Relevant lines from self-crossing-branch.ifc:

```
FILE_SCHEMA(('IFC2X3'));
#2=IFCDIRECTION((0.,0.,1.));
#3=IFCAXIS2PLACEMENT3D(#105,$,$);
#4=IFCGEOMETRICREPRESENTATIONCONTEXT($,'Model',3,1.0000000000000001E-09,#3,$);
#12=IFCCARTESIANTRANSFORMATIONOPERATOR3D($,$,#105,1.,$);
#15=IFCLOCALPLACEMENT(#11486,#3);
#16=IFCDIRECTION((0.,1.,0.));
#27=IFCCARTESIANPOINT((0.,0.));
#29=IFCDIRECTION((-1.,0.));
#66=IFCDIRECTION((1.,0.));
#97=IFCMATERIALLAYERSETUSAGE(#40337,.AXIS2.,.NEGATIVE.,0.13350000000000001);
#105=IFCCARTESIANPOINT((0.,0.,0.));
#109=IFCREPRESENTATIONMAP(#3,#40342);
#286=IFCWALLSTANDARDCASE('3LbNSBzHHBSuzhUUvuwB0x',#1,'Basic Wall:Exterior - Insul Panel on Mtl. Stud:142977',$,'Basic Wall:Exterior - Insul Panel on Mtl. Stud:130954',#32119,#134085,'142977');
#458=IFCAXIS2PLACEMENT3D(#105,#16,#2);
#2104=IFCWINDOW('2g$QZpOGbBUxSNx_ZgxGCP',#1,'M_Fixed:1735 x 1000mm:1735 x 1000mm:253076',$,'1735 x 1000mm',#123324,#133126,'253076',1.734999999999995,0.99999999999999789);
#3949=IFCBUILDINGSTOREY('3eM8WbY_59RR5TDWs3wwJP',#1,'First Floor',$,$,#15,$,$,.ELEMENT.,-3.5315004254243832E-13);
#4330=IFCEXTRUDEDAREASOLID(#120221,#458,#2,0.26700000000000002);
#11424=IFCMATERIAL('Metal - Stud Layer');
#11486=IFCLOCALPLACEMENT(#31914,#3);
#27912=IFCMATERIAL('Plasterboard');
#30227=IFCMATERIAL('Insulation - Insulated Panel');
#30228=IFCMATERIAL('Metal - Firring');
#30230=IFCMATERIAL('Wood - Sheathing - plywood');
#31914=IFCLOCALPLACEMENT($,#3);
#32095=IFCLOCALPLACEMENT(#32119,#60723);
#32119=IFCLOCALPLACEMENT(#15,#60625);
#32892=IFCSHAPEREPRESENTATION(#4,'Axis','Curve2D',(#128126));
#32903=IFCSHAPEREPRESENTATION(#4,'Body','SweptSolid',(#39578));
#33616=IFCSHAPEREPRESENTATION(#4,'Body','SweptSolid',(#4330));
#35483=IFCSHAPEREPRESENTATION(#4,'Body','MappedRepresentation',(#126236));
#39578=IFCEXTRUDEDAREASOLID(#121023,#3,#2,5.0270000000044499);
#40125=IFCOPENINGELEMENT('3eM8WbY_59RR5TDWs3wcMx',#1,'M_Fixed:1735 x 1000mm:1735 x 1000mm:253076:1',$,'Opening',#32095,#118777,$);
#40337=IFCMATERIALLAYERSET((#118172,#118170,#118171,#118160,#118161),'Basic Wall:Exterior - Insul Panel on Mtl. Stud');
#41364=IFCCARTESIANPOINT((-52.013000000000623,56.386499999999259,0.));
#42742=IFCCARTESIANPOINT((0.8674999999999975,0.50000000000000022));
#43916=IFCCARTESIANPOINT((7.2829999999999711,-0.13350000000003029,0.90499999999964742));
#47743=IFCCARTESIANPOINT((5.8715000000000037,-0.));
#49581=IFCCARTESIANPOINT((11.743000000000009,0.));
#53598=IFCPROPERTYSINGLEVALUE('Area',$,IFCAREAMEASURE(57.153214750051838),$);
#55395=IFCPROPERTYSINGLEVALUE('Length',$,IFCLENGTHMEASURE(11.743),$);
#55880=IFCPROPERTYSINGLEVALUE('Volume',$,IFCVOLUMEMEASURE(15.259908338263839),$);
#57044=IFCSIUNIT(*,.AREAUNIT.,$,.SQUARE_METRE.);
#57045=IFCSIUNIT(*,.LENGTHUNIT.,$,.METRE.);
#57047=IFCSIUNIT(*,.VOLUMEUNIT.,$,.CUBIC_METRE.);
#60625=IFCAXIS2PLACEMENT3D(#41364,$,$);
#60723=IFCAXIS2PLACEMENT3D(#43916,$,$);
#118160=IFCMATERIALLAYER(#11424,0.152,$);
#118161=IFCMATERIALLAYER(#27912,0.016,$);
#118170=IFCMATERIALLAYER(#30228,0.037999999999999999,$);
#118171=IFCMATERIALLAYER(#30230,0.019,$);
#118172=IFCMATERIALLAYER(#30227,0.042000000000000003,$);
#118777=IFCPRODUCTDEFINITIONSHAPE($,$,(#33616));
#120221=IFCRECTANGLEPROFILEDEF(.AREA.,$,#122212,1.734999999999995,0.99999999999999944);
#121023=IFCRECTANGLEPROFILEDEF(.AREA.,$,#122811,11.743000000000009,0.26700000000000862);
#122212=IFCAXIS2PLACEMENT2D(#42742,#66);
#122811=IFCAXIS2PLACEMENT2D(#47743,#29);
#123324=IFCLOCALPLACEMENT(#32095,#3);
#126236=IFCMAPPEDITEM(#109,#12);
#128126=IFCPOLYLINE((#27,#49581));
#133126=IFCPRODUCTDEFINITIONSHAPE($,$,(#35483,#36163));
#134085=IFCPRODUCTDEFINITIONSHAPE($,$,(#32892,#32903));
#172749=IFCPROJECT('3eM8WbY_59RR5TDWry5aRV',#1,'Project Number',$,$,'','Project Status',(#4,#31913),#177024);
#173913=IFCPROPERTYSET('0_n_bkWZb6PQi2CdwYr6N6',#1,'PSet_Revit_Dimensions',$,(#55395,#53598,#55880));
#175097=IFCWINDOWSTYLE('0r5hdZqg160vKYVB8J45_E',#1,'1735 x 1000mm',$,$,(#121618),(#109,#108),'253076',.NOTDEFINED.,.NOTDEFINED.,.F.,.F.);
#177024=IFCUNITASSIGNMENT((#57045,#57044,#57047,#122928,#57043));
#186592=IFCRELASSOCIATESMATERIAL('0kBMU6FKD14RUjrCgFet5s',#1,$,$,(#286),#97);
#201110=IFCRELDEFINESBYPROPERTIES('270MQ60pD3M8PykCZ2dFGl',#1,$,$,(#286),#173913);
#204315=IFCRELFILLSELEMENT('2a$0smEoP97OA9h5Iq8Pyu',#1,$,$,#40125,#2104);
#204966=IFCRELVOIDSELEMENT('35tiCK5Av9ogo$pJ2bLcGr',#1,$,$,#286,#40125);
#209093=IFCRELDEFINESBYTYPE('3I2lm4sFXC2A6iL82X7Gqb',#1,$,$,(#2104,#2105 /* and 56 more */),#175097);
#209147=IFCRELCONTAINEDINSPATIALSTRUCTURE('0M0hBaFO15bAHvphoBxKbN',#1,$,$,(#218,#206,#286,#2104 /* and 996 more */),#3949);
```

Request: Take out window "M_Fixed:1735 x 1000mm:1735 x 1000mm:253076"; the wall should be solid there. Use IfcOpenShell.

```python
import ifcopenshell
import ifcopenshell.api.feature
import ifcopenshell.api.pset
import ifcopenshell.api.root
import ifcopenshell.geom
import ifcopenshell.util.element
import ifcopenshell.util.shape
import ifcopenshell.util.unit

model = ifcopenshell.open("self-crossing-branch.ifc")
area_scale = ifcopenshell.util.unit.calculate_unit_scale(model, "AREAUNIT")
volume_scale = ifcopenshell.util.unit.calculate_unit_scale(model, "VOLUMEUNIT")
settings = ifcopenshell.geom.settings()


def volume(element):
    """Net volume in cubic metres, openings subtracted."""
    shape = ifcopenshell.geom.create_shape(settings, element)
    return ifcopenshell.util.shape.get_volume(shape.geometry)


window = model.by_guid("2g$QZpOGbBUxSNx_ZgxGCP")
opening = window.FillsVoids[0].RelatingOpeningElement
wall = opening.VoidsElements[0].RelatingBuildingElement
before = volume(wall)

ifcopenshell.api.root.remove_product(model, product=window)
ifcopenshell.api.feature.remove_feature(model, feature=opening)

after = volume(wall)
thickness = 0.267  # wall thickness in metres

# Update the wall's stored quantities.
pset = model.by_id(ifcopenshell.util.element.get_pset(wall, "PSet_Revit_Dimensions", should_inherit=False)["id"])
ifcopenshell.api.pset.edit_pset(model, pset=pset, properties={
    "Area": model.create_entity("IfcAreaMeasure", after / thickness / area_scale),
    "Volume": model.create_entity("IfcVolumeMeasure", after / volume_scale),
})

print(f"wall volume {before:.3f} -> {after:.3f} m3")

model.write("self-crossing-branch_updated.ifc")
```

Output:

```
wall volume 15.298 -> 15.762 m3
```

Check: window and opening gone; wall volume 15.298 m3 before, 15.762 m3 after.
